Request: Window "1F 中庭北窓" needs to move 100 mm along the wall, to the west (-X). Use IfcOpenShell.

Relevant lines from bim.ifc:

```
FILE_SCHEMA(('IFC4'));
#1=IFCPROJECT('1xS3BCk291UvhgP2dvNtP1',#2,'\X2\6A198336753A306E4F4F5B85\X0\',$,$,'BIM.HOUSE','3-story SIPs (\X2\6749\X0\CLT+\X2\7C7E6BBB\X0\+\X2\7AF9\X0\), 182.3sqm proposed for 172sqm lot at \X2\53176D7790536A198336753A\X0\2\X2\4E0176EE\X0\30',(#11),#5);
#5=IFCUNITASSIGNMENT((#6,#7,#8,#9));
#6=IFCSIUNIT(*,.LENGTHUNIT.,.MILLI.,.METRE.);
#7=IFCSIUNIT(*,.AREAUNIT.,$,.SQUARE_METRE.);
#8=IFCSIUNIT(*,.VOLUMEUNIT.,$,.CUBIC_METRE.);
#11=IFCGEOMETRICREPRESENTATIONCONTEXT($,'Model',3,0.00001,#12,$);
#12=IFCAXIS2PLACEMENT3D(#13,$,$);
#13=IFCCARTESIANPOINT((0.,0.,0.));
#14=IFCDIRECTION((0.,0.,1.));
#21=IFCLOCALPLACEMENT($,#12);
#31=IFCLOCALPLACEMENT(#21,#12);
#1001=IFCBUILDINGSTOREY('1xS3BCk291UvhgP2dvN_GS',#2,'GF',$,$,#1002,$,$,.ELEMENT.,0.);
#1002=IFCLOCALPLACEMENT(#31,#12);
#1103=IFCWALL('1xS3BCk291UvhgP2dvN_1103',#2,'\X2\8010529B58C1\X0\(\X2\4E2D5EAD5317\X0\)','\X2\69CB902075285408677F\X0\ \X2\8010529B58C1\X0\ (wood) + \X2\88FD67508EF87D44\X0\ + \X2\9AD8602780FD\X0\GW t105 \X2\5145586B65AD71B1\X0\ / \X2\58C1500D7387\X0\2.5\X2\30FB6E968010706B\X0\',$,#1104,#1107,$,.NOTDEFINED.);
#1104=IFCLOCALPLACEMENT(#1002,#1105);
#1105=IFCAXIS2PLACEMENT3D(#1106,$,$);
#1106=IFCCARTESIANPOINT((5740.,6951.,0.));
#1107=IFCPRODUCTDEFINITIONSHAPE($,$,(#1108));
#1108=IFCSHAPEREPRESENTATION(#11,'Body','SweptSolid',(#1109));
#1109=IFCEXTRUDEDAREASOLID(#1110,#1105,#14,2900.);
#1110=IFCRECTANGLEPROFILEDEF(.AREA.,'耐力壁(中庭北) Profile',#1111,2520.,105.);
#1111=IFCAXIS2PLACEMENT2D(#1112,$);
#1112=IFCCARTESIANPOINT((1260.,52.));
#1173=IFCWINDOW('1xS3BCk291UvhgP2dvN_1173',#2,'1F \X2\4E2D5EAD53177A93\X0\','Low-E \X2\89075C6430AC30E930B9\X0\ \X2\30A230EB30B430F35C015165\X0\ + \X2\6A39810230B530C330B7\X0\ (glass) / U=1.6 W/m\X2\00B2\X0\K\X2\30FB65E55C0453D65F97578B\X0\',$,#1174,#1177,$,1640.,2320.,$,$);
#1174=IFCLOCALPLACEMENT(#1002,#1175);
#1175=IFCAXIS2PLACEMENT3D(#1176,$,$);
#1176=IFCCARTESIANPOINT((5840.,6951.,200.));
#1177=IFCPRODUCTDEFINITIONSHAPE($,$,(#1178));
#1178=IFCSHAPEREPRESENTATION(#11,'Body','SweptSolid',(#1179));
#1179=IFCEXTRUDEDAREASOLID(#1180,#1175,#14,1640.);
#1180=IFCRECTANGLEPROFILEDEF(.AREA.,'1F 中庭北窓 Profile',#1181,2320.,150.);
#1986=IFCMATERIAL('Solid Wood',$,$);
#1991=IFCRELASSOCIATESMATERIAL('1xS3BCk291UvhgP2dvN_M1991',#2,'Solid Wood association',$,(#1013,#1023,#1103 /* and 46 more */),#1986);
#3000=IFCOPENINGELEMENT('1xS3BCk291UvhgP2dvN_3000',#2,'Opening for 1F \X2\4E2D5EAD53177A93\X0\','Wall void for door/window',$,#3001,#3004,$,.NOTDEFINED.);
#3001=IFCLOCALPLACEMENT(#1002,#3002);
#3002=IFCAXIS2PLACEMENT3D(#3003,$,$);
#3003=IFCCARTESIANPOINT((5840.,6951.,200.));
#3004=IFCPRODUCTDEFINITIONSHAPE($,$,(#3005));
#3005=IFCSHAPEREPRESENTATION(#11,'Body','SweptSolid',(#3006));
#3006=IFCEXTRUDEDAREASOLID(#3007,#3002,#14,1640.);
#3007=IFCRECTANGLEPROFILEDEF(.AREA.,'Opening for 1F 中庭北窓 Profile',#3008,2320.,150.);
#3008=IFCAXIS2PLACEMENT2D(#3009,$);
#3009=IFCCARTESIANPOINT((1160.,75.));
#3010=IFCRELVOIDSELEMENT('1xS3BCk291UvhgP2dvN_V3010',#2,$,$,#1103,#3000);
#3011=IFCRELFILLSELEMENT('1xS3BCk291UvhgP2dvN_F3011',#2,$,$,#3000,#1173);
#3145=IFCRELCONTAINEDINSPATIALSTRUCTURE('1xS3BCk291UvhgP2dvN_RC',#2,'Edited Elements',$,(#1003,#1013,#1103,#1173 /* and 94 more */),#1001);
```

```python
import ifcopenshell
import ifcopenshell.api.geometry
import ifcopenshell.util.placement
import ifcopenshell.util.unit

model = ifcopenshell.open("bim.ifc")
unit_scale = ifcopenshell.util.unit.calculate_unit_scale(model)

window = model.by_guid("1xS3BCk291UvhgP2dvN_1173")
opening = window.FillsVoids[0].RelatingOpeningElement
wall = opening.VoidsElements[0].RelatingBuildingElement

wall_matrix = ifcopenshell.util.placement.get_local_placement(wall.ObjectPlacement)
shift = wall_matrix[:3, 0] * -0.1 / unit_scale
before = ifcopenshell.util.placement.get_local_placement(window.ObjectPlacement)[:3, 3].copy()

# The window is not placed relative to its opening, so move both.
for product in (opening, window):
    matrix = ifcopenshell.util.placement.get_local_placement(product.ObjectPlacement)
    matrix[:3, 3] += shift
    ifcopenshell.api.geometry.edit_object_placement(model, product=product, matrix=matrix, is_si=False)

after = ifcopenshell.util.placement.get_local_placement(window.ObjectPlacement)[:3, 3]
print("window moved by", (after - before).round(3) + 0.0)

model.write("bim_rev.ifc")
```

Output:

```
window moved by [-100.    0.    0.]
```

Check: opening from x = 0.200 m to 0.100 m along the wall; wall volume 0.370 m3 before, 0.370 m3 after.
